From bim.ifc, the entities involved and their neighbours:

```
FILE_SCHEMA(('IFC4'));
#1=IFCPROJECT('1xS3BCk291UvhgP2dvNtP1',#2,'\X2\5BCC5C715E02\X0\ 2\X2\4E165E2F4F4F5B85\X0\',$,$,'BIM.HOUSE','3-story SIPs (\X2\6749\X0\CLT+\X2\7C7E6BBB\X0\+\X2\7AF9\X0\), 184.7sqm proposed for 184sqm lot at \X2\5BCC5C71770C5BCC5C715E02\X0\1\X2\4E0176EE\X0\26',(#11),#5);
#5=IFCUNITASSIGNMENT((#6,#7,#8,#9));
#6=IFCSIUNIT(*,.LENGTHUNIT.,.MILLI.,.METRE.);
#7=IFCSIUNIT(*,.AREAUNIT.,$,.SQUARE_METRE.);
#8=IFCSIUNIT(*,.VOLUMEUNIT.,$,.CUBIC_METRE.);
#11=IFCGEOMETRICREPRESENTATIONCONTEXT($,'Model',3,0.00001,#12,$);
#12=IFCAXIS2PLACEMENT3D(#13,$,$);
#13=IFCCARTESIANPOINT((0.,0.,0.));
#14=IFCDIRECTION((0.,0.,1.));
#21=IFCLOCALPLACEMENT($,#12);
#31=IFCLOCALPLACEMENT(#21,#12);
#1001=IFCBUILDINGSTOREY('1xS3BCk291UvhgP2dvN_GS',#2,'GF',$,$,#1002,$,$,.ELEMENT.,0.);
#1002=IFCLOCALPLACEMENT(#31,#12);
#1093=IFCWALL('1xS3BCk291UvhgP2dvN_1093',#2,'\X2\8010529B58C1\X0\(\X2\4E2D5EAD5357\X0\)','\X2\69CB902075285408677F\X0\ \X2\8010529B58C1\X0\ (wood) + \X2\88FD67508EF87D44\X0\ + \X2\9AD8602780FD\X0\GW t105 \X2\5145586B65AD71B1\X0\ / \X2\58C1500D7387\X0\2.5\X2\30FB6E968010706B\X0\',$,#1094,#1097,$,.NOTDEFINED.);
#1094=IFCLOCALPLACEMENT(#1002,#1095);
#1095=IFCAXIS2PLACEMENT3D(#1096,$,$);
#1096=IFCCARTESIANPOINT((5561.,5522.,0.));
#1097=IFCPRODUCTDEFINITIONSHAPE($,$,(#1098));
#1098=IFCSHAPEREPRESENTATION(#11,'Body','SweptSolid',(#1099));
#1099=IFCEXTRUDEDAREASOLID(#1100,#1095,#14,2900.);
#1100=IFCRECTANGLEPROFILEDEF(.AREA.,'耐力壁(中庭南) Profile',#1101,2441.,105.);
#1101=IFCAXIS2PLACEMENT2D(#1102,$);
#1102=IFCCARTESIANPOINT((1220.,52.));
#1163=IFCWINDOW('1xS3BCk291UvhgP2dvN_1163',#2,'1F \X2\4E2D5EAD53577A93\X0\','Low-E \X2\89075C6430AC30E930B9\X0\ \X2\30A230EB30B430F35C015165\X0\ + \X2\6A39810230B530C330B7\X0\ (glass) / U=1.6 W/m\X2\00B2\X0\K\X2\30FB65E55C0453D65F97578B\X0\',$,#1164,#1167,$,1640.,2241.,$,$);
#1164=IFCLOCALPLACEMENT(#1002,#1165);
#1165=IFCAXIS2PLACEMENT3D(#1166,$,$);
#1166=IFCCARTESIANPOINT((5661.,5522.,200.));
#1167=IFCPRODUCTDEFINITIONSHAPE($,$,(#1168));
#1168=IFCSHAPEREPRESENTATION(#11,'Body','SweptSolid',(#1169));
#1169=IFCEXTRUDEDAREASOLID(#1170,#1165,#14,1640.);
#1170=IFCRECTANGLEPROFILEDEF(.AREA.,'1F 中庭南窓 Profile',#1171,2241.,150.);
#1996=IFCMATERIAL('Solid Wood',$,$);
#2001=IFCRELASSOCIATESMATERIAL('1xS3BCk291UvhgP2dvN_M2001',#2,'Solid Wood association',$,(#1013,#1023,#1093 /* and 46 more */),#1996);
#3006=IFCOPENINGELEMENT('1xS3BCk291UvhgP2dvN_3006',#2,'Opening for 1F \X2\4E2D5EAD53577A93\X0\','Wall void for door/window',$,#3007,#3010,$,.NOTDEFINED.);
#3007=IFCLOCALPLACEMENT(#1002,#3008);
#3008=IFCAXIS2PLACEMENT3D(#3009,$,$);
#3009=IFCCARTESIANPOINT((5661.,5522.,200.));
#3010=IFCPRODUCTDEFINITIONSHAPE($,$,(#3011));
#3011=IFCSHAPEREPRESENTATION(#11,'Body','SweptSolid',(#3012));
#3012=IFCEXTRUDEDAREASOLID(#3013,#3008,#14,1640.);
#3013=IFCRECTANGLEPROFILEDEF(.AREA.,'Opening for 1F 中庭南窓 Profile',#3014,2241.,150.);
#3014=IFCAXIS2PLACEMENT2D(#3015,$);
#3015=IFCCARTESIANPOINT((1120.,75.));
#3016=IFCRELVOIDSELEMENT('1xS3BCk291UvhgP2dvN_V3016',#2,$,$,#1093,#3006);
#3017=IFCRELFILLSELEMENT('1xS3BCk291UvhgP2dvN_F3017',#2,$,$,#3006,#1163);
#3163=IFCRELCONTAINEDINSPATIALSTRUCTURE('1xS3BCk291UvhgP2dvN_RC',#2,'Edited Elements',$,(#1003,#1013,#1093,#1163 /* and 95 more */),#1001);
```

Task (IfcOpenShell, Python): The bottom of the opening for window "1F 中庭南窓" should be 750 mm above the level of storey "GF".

```python
import numpy as np
import ifcopenshell
import ifcopenshell.api.geometry
import ifcopenshell.geom
import ifcopenshell.util.element
import ifcopenshell.util.placement
import ifcopenshell.util.shape
import ifcopenshell.util.unit

model = ifcopenshell.open("bim.ifc")
unit_scale = ifcopenshell.util.unit.calculate_unit_scale(model)

window = model.by_guid("1xS3BCk291UvhgP2dvN_1163")
opening = window.FillsVoids[0].RelatingOpeningElement
storey = ifcopenshell.util.element.get_container(window, ifc_class="IfcBuildingStorey")
level = ifcopenshell.util.placement.get_local_placement(storey.ObjectPlacement)[2, 3]

# The opening's origin need not be at the sill, so measure its lowest point.
shape = ifcopenshell.geom.create_shape(ifcopenshell.geom.settings(), opening)
bottom = ifcopenshell.util.shape.get_shape_bottom_elevation(shape, shape.geometry) / unit_scale
dz = level + 0.75 / unit_scale - bottom

shift = np.array([0.0, 0.0, dz])
# The window is not placed relative to its opening, so move both.
for product in (opening, window):
    matrix = ifcopenshell.util.placement.get_local_placement(product.ObjectPlacement)
    matrix[:3, 3] += shift
    ifcopenshell.api.geometry.edit_object_placement(model, product=product, matrix=matrix, is_si=False)

print(f"moved by {dz * unit_scale:+.3f} m")

model.write("bim_updated.ifc")
```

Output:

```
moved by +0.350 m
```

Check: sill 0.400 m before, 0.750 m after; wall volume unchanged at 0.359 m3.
